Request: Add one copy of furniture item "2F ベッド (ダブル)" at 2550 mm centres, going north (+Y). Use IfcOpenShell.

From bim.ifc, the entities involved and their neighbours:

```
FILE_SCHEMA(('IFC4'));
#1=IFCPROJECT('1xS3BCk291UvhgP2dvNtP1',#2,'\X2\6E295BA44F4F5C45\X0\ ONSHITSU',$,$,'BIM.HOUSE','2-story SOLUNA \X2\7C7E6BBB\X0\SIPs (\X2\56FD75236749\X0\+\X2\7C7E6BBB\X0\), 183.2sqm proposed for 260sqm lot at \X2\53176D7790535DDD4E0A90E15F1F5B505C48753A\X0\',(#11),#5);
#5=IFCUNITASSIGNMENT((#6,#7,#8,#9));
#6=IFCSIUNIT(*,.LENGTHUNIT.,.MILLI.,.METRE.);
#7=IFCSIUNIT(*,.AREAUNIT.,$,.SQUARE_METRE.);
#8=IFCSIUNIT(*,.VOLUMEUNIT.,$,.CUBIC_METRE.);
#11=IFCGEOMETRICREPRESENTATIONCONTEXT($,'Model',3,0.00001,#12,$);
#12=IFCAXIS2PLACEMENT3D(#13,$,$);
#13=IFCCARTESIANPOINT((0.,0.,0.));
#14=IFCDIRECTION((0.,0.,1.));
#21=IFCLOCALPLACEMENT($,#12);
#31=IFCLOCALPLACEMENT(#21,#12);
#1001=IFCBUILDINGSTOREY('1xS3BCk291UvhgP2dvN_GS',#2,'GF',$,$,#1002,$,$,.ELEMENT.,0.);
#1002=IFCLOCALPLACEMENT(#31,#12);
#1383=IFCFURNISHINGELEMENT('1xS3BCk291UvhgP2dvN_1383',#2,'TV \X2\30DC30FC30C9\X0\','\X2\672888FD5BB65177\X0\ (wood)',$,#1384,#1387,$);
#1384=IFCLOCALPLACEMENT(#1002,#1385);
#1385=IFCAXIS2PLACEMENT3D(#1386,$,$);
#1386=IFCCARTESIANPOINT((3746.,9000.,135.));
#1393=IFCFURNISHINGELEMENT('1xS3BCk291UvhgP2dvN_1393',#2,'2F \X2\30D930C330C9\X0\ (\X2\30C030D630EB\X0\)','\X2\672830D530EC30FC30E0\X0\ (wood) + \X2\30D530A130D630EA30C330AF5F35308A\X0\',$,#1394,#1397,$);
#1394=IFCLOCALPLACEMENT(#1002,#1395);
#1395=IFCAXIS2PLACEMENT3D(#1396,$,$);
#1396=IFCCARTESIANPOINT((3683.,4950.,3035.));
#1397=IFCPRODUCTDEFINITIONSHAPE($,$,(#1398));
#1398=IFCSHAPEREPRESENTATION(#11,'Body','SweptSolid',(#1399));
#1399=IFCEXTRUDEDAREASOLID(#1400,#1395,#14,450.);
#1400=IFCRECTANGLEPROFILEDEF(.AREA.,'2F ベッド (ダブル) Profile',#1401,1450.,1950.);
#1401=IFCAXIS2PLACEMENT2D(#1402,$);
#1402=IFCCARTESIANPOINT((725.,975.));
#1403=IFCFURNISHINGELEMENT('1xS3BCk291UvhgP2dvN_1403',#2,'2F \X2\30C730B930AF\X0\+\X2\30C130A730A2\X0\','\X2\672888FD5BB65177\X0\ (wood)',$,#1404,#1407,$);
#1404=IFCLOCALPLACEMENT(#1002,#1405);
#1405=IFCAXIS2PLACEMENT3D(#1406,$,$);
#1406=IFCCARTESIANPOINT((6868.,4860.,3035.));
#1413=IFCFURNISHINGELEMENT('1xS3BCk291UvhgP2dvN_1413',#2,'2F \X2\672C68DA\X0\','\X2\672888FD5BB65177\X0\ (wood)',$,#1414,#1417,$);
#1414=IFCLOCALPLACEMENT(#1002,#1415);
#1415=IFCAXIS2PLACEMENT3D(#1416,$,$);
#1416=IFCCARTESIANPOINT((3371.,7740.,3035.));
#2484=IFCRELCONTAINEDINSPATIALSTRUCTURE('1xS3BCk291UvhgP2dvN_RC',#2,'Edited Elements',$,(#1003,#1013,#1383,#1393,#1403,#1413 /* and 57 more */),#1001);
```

```python
import numpy as np
import ifcopenshell
import ifcopenshell.api.geometry
import ifcopenshell.api.root
import ifcopenshell.util.element
import ifcopenshell.util.placement
import ifcopenshell.util.unit

model = ifcopenshell.open("bim.ifc")
unit_scale = ifcopenshell.util.unit.calculate_unit_scale(model)


def reuse_history(source, copy):
    """copy_class also copies each property set's owner history, people and application; keep the originals."""
    for rel in copy.IsDefinedBy:
        if rel.is_a("IfcRelDefinesByProperties") and (history := rel.RelatingPropertyDefinition.OwnerHistory):
            rel.RelatingPropertyDefinition.OwnerHistory = source.OwnerHistory
            ifcopenshell.util.element.remove_deep2(model, history)


source = model.by_guid("1xS3BCk291UvhgP2dvN_1393")
base = ifcopenshell.util.placement.get_local_placement(source.ObjectPlacement)
step = np.array([0.0, 1.0, 0.0]) * 2.55 / unit_scale

for i in range(1, 2):
    copy = ifcopenshell.api.root.copy_class(model, product=source)
    copy.Representation = ifcopenshell.util.element.copy_deep(
        model, source.Representation, exclude=["IfcGeometricRepresentationContext", "IfcRepresentationMap"]
    )
    reuse_history(source, copy)
    matrix = base.copy()
    matrix[:3, 3] += i * step
    print("added at", matrix[:3, 3].round(3) + 0.0)
    ifcopenshell.api.geometry.edit_object_placement(model, product=copy, matrix=matrix, is_si=False)

model.write("bim_updated.ifc")
```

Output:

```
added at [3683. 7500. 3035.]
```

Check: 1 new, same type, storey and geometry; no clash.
